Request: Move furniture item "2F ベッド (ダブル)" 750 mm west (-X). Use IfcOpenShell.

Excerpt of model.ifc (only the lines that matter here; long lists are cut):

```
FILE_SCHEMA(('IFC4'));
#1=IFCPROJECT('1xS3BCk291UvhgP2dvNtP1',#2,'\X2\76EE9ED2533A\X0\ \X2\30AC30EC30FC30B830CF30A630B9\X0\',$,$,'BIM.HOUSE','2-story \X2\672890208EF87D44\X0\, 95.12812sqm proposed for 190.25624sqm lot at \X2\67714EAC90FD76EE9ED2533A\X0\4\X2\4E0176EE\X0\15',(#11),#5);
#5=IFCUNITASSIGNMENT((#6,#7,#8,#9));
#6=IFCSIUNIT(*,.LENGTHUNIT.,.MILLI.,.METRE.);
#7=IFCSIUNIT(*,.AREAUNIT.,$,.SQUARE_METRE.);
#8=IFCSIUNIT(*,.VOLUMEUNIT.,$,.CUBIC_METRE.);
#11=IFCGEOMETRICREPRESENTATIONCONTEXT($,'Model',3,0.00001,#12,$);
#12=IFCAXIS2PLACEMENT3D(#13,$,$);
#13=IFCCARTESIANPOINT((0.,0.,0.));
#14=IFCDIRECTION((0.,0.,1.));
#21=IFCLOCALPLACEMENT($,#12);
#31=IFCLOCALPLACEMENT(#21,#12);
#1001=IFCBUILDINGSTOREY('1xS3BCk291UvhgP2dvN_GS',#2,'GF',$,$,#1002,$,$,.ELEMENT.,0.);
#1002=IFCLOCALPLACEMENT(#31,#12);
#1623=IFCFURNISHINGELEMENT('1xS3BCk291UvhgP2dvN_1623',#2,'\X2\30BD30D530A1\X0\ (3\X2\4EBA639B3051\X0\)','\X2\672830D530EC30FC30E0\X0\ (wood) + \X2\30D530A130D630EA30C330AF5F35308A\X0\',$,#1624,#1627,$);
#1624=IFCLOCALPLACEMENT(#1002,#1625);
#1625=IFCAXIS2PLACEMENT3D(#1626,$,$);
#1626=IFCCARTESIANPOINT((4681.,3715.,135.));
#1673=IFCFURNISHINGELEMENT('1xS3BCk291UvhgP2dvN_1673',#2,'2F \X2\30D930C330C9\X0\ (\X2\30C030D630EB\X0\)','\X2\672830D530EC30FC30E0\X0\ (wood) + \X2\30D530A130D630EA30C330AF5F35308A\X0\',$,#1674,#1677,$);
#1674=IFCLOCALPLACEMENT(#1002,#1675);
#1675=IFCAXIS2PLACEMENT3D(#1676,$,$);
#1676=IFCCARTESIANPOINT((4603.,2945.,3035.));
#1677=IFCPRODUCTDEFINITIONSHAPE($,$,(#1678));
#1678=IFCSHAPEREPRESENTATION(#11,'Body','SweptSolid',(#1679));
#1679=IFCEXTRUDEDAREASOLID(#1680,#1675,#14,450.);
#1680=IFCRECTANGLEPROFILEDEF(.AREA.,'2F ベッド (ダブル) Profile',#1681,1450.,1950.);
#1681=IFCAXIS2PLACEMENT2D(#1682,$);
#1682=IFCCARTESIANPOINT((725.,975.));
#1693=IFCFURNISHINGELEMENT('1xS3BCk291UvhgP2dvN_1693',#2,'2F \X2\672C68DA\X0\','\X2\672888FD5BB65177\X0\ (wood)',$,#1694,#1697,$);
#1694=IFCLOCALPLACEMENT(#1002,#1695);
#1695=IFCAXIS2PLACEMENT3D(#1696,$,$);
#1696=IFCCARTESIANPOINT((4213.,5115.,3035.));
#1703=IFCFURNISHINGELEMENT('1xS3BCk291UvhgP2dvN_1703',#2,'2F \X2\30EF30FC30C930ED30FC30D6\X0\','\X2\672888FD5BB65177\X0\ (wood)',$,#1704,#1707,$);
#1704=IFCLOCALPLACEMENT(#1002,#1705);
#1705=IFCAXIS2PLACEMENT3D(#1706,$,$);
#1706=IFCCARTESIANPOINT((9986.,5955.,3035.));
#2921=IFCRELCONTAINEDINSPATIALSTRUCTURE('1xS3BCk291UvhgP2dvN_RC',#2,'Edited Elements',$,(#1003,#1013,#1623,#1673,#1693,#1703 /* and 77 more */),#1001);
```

```python
import ifcopenshell
import ifcopenshell.api.geometry
import ifcopenshell.util.placement
import ifcopenshell.util.unit

model = ifcopenshell.open("model.ifc")
unit_scale = ifcopenshell.util.unit.calculate_unit_scale(model)

item = model.by_id(1673)
matrix = ifcopenshell.util.placement.get_local_placement(item.ObjectPlacement)
matrix[0, 3] -= 0.75 / unit_scale
ifcopenshell.api.geometry.edit_object_placement(model, product=item, matrix=matrix, is_si=False)

print(ifcopenshell.util.placement.get_local_placement(item.ObjectPlacement).round(3) + 0.0)

model.write("model_rev.ifc")
```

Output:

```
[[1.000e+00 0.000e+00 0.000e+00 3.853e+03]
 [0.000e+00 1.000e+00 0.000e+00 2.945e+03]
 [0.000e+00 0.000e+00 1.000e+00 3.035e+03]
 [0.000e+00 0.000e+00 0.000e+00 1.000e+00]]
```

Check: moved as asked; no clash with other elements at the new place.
